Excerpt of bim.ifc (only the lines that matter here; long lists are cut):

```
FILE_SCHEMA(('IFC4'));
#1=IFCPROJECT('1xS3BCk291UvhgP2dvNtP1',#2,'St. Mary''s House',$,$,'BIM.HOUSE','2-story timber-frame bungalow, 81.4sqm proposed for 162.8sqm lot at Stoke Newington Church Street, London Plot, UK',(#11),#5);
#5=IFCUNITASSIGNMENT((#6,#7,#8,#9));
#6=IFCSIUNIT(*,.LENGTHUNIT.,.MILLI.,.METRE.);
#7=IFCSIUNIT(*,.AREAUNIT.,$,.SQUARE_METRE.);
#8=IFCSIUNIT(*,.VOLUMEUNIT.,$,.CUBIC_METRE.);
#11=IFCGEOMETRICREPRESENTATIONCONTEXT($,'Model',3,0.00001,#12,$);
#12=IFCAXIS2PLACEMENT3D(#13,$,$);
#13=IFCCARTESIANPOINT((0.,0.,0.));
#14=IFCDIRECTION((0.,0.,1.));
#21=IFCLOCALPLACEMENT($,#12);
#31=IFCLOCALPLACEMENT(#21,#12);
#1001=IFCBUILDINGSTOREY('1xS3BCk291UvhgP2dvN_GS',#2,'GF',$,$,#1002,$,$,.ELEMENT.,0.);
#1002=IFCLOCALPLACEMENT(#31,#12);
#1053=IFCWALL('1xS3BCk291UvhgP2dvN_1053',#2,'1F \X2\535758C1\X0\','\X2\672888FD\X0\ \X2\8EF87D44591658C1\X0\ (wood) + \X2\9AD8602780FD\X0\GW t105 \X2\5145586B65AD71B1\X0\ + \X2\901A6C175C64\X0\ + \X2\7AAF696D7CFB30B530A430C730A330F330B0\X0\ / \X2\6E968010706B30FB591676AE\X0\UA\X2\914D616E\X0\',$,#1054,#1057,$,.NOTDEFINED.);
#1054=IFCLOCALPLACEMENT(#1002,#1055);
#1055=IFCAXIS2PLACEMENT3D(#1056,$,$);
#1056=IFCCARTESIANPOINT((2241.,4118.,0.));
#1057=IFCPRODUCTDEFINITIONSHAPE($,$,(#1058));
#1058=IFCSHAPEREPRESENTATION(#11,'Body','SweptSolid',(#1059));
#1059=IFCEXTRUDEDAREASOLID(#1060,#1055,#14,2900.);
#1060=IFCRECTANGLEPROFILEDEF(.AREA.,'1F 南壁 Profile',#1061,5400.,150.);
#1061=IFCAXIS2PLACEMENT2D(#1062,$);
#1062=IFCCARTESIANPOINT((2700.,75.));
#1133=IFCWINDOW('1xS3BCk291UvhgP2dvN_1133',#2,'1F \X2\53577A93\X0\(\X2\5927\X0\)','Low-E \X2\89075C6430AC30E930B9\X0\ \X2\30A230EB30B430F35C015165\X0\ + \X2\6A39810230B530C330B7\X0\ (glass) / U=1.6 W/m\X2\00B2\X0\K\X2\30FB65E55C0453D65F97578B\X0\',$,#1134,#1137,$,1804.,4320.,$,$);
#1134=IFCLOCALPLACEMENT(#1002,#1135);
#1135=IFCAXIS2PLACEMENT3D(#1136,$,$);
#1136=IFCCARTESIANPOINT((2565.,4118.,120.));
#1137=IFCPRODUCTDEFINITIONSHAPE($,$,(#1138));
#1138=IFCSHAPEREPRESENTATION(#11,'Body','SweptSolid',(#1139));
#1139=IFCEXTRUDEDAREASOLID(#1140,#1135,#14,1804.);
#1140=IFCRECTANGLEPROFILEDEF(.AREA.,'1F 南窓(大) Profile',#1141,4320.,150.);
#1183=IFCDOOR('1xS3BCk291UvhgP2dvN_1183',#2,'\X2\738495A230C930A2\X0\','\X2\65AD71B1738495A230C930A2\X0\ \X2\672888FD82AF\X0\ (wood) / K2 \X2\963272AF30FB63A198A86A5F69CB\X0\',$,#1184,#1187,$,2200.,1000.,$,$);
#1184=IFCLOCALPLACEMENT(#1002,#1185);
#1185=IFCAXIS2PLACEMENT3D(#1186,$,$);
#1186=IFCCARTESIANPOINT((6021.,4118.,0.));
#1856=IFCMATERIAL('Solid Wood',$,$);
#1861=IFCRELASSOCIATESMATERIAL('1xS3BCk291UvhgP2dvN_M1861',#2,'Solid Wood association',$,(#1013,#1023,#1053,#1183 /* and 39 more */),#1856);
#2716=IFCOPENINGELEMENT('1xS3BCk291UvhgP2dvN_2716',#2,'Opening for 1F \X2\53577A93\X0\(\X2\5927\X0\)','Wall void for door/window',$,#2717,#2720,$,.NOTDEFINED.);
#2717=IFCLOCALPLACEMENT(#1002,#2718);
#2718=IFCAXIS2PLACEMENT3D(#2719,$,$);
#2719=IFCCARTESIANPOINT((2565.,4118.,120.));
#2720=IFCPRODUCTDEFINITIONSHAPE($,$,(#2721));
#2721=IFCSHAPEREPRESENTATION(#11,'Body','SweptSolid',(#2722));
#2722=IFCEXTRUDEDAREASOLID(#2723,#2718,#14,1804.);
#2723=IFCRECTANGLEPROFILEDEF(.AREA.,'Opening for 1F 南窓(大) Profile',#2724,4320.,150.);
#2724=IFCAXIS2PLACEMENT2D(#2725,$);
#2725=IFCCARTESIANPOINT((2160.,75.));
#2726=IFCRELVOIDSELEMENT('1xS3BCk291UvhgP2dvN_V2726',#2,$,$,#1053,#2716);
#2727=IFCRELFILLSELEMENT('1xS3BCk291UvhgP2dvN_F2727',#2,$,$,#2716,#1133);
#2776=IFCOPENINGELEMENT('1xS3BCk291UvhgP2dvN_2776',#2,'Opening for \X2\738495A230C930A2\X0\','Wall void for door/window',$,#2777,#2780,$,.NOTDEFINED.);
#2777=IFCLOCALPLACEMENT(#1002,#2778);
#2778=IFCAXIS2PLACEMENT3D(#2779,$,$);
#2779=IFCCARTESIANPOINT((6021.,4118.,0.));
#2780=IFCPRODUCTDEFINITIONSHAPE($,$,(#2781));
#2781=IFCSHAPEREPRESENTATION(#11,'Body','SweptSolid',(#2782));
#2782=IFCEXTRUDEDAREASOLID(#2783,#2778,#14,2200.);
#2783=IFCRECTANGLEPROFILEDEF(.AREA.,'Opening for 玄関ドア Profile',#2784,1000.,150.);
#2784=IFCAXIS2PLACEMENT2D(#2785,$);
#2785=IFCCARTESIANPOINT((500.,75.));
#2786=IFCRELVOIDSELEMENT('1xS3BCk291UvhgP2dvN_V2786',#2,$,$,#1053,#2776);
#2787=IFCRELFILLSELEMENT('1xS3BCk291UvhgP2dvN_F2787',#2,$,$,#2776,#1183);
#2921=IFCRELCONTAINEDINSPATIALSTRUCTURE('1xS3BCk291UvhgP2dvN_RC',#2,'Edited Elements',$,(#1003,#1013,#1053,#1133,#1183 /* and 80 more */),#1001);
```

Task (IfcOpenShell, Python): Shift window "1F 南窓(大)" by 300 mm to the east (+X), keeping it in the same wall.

```python
import ifcopenshell
import ifcopenshell.api.geometry
import ifcopenshell.util.placement

model = ifcopenshell.open("bim.ifc")

window = model.by_guid("1xS3BCk291UvhgP2dvN_1133")
opening = window.FillsVoids[0].RelatingOpeningElement
wall = opening.VoidsElements[0].RelatingBuildingElement

wall_matrix = ifcopenshell.util.placement.get_local_placement(wall.ObjectPlacement)
shift = wall_matrix[:3, 0] * 300.0
before = ifcopenshell.util.placement.get_local_placement(window.ObjectPlacement)[:3, 3].copy()

# The window is not placed relative to its opening, so move both.
for product in (opening, window):
    matrix = ifcopenshell.util.placement.get_local_placement(product.ObjectPlacement)
    matrix[:3, 3] += shift
    ifcopenshell.api.geometry.edit_object_placement(model, product=product, matrix=matrix, is_si=False)

after = ifcopenshell.util.placement.get_local_placement(window.ObjectPlacement)[:3, 3]
print("window moved by", (after - before).round(3) + 0.0)

model.write("bim_updated.ifc")
```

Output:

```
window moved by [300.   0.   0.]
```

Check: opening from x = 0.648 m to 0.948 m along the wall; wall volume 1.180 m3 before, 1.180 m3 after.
